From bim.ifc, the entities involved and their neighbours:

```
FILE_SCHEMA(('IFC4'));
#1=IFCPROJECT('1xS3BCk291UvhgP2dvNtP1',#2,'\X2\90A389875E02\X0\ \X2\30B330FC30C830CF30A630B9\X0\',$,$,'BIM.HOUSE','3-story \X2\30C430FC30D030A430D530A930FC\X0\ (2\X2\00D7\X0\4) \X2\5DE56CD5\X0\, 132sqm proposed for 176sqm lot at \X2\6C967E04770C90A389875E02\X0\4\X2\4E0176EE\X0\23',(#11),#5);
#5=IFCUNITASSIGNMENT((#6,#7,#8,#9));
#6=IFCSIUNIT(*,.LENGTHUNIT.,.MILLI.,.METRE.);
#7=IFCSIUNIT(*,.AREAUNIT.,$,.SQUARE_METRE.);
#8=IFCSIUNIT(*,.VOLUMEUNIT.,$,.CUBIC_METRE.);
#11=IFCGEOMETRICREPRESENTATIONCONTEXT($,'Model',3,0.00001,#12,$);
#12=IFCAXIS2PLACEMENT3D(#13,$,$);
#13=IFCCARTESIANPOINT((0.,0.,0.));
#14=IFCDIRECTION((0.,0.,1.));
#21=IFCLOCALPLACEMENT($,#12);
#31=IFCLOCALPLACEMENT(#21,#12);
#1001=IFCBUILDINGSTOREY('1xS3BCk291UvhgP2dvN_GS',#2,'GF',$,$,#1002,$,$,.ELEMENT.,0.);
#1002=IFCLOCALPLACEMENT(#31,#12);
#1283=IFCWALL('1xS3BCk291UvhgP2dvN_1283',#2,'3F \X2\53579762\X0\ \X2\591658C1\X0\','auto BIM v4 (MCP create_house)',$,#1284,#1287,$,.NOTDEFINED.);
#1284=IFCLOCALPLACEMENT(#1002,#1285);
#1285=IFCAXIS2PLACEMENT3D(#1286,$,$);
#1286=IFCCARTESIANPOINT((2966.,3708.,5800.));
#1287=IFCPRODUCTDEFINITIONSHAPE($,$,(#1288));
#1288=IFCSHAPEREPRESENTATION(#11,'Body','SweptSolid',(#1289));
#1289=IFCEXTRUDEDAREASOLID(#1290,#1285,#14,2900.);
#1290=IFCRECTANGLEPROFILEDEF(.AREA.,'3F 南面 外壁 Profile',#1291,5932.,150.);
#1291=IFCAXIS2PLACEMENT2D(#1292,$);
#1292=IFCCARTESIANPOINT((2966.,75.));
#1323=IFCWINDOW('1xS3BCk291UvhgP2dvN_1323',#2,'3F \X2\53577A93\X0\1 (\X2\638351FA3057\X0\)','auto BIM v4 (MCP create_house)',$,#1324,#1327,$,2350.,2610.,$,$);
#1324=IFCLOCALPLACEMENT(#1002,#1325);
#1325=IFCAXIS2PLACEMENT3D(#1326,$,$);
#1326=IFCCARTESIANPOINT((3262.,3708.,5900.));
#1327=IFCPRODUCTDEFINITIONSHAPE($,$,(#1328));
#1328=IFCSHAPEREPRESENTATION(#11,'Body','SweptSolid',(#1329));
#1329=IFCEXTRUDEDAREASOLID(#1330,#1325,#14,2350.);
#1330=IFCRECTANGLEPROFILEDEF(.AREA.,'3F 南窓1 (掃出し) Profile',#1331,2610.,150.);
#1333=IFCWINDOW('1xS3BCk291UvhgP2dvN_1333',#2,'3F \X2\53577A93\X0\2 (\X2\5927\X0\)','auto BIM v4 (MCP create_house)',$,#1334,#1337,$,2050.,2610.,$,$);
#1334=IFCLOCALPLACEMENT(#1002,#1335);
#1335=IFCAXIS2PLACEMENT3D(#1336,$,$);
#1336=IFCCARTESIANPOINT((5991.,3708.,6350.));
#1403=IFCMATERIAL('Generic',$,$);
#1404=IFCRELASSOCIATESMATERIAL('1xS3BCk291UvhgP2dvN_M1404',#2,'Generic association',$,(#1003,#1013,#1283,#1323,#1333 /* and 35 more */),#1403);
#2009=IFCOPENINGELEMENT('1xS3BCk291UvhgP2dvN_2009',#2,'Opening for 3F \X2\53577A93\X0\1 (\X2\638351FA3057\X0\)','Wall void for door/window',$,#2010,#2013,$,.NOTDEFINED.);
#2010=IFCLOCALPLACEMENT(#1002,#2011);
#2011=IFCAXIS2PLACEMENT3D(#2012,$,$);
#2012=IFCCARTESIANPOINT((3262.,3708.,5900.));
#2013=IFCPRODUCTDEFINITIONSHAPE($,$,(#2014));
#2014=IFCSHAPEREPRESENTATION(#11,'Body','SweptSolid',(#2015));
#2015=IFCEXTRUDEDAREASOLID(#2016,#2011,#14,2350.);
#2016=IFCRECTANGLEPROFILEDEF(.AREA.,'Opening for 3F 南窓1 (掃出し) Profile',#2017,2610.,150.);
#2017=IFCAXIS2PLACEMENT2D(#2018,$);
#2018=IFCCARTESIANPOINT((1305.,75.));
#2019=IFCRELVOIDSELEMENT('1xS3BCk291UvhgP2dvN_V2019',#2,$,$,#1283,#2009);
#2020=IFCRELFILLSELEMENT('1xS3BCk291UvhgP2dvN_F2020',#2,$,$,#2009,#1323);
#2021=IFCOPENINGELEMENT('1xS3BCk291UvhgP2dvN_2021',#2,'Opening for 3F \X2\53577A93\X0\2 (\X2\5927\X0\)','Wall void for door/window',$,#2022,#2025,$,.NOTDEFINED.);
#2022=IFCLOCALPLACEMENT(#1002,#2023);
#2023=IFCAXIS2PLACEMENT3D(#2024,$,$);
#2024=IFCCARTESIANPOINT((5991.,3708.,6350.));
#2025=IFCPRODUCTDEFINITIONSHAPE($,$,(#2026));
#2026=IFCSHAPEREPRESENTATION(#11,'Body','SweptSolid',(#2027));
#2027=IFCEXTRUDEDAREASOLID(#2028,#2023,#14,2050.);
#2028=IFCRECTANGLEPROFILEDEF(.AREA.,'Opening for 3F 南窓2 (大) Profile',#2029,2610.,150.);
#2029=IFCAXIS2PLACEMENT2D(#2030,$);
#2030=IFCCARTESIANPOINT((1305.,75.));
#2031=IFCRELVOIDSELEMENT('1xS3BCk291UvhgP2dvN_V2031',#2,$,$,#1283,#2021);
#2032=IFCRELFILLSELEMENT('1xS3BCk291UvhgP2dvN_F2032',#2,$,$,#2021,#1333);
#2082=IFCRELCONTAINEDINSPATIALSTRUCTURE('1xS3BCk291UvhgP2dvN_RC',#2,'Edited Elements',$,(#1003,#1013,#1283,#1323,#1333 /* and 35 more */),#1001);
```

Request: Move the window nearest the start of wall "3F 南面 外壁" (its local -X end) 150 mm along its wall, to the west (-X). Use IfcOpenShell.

```python
import ifcopenshell
import ifcopenshell.api.geometry
import ifcopenshell.util.placement
import ifcopenshell.util.unit

model = ifcopenshell.open("bim.ifc")
unit_scale = ifcopenshell.util.unit.calculate_unit_scale(model)

window = model.by_guid("1xS3BCk291UvhgP2dvN_1323")
opening = window.FillsVoids[0].RelatingOpeningElement
wall = opening.VoidsElements[0].RelatingBuildingElement

wall_matrix = ifcopenshell.util.placement.get_local_placement(wall.ObjectPlacement)
shift = wall_matrix[:3, 0] * -0.15 / unit_scale
before = ifcopenshell.util.placement.get_local_placement(window.ObjectPlacement)[:3, 3].copy()

# The window is not placed relative to its opening, so move both.
for product in (opening, window):
    matrix = ifcopenshell.util.placement.get_local_placement(product.ObjectPlacement)
    matrix[:3, 3] += shift
    ifcopenshell.api.geometry.edit_object_placement(model, product=product, matrix=matrix, is_si=False)

after = ifcopenshell.util.placement.get_local_placement(window.ObjectPlacement)[:3, 3]
print("window moved by", (after - before).round(3) + 0.0)

model.write("bim_updated.ifc")
```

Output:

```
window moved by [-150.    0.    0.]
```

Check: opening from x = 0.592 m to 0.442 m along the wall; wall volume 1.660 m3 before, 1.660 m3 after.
